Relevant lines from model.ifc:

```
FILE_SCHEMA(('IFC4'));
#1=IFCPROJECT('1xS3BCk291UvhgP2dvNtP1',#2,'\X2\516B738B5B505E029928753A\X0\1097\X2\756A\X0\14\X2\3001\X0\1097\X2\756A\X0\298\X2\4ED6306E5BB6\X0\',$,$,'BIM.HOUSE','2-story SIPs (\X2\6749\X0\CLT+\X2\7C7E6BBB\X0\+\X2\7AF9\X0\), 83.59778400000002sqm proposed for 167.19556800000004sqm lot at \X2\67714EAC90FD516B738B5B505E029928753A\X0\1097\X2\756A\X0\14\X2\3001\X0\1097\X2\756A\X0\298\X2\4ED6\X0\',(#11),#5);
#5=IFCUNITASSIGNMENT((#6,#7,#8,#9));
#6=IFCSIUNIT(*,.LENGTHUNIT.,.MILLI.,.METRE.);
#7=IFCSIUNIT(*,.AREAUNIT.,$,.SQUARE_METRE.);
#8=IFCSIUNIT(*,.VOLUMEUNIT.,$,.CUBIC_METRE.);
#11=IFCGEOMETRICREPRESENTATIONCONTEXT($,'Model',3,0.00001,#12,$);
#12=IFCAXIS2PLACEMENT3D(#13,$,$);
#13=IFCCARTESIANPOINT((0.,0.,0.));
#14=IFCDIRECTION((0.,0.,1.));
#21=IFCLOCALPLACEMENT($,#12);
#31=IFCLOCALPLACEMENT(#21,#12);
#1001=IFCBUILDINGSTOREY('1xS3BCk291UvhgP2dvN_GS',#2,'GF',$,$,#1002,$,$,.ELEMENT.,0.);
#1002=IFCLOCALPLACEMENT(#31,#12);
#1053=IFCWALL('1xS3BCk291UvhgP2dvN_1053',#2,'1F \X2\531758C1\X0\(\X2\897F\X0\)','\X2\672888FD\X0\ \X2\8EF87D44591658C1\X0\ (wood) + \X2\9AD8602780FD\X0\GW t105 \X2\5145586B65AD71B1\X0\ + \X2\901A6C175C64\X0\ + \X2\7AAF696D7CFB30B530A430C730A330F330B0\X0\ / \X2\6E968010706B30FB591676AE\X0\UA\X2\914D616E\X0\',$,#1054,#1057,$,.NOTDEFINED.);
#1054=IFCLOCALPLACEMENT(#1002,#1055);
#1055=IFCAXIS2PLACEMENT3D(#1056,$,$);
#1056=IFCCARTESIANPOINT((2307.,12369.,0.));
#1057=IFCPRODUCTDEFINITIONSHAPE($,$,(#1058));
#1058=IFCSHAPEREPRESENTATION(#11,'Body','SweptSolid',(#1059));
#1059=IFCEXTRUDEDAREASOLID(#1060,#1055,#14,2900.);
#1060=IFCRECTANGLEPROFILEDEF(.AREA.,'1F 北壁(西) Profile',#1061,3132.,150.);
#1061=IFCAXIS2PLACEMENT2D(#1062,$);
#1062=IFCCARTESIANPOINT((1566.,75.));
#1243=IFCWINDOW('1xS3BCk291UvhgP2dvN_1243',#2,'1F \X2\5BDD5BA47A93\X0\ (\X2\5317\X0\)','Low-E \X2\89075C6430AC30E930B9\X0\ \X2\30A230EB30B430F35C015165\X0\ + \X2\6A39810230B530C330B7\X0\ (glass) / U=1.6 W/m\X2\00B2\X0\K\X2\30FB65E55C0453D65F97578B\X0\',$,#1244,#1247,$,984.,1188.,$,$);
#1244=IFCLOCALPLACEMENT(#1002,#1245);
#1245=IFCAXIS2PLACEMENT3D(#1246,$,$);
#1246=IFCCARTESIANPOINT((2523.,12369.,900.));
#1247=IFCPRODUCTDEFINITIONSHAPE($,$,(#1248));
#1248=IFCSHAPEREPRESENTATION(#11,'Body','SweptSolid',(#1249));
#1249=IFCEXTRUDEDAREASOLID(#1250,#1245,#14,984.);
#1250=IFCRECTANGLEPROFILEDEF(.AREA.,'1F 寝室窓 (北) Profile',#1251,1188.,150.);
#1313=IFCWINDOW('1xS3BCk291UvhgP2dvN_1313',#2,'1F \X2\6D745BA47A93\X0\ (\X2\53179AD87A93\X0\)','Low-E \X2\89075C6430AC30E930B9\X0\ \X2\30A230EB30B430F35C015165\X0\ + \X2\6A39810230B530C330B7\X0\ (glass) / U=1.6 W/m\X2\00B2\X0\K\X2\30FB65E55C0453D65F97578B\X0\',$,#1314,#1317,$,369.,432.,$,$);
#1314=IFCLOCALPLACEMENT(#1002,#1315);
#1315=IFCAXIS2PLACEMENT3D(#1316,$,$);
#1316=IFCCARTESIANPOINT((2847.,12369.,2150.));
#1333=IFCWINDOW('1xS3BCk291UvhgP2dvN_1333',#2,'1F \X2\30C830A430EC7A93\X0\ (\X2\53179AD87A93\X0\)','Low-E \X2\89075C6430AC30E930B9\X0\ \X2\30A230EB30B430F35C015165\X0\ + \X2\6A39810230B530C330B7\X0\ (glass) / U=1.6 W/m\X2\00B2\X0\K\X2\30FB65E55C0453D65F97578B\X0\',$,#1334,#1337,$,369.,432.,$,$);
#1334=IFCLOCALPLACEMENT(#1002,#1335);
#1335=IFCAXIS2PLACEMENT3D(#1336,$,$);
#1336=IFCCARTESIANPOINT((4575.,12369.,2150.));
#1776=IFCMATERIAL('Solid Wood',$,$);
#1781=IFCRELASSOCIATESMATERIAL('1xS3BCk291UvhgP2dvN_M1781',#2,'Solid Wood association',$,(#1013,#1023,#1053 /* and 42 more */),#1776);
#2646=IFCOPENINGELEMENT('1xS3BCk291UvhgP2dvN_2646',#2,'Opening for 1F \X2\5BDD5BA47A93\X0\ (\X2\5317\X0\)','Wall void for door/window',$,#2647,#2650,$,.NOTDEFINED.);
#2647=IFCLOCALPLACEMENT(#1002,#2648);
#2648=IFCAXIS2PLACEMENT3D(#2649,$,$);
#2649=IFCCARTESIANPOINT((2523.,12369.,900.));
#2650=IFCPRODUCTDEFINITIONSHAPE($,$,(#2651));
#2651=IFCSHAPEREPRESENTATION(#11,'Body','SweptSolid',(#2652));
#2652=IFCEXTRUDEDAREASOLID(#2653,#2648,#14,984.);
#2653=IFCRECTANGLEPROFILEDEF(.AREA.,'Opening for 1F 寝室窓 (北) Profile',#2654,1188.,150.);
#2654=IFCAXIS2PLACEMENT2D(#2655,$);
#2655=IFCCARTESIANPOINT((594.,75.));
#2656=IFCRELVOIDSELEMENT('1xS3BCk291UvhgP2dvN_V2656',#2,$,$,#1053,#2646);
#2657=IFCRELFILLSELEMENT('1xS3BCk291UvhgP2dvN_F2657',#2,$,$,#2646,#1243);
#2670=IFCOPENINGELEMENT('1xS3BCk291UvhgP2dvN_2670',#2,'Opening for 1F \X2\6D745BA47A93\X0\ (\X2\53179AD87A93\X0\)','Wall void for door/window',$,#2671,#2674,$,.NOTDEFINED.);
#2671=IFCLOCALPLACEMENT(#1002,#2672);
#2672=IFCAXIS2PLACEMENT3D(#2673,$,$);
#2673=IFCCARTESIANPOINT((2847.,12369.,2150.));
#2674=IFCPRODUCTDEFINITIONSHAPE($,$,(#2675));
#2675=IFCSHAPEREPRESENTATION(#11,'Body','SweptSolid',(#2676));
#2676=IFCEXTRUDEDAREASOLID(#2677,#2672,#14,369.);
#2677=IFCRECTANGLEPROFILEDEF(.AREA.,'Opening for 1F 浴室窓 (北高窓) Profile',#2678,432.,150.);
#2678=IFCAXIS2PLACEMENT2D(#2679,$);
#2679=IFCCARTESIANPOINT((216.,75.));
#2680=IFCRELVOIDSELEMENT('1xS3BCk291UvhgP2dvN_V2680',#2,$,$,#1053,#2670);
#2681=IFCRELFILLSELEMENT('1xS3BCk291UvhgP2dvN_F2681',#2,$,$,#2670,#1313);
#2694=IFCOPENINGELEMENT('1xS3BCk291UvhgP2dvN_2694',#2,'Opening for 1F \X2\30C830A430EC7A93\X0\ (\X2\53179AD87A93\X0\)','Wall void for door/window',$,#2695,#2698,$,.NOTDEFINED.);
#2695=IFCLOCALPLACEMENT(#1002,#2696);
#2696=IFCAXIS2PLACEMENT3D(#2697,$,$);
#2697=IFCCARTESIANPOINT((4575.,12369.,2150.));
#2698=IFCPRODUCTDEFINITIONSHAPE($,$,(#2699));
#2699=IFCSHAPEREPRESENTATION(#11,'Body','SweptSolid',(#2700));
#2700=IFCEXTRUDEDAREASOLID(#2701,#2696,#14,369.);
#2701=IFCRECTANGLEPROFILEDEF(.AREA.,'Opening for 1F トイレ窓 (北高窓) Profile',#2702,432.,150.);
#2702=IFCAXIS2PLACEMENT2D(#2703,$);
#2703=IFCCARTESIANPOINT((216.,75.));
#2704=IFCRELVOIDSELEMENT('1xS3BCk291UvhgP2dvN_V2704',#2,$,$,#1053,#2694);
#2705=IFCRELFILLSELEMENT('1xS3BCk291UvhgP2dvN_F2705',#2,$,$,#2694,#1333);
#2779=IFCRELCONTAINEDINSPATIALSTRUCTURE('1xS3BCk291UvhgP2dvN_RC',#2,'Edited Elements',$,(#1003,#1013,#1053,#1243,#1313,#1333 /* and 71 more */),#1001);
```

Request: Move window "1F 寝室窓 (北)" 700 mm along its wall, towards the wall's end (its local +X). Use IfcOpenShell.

```python
import ifcopenshell
import ifcopenshell.api.geometry
import ifcopenshell.util.placement
import ifcopenshell.util.unit

model = ifcopenshell.open("model.ifc")
unit_scale = ifcopenshell.util.unit.calculate_unit_scale(model)

window = model.by_id(1243)
opening = window.FillsVoids[0].RelatingOpeningElement
wall = opening.VoidsElements[0].RelatingBuildingElement

wall_matrix = ifcopenshell.util.placement.get_local_placement(wall.ObjectPlacement)
shift = wall_matrix[:3, 0] * 0.7 / unit_scale
before = ifcopenshell.util.placement.get_local_placement(window.ObjectPlacement)[:3, 3].copy()

# The window is not placed relative to its opening, so move both.
for product in (opening, window):
    matrix = ifcopenshell.util.placement.get_local_placement(product.ObjectPlacement)
    matrix[:3, 3] += shift
    ifcopenshell.api.geometry.edit_object_placement(model, product=product, matrix=matrix, is_si=False)

after = ifcopenshell.util.placement.get_local_placement(window.ObjectPlacement)[:3, 3]
print("window moved by", (after - before).round(3) + 0.0)

model.write("model-out.ifc")
```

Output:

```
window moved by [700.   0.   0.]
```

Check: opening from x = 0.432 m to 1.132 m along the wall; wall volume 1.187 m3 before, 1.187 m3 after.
